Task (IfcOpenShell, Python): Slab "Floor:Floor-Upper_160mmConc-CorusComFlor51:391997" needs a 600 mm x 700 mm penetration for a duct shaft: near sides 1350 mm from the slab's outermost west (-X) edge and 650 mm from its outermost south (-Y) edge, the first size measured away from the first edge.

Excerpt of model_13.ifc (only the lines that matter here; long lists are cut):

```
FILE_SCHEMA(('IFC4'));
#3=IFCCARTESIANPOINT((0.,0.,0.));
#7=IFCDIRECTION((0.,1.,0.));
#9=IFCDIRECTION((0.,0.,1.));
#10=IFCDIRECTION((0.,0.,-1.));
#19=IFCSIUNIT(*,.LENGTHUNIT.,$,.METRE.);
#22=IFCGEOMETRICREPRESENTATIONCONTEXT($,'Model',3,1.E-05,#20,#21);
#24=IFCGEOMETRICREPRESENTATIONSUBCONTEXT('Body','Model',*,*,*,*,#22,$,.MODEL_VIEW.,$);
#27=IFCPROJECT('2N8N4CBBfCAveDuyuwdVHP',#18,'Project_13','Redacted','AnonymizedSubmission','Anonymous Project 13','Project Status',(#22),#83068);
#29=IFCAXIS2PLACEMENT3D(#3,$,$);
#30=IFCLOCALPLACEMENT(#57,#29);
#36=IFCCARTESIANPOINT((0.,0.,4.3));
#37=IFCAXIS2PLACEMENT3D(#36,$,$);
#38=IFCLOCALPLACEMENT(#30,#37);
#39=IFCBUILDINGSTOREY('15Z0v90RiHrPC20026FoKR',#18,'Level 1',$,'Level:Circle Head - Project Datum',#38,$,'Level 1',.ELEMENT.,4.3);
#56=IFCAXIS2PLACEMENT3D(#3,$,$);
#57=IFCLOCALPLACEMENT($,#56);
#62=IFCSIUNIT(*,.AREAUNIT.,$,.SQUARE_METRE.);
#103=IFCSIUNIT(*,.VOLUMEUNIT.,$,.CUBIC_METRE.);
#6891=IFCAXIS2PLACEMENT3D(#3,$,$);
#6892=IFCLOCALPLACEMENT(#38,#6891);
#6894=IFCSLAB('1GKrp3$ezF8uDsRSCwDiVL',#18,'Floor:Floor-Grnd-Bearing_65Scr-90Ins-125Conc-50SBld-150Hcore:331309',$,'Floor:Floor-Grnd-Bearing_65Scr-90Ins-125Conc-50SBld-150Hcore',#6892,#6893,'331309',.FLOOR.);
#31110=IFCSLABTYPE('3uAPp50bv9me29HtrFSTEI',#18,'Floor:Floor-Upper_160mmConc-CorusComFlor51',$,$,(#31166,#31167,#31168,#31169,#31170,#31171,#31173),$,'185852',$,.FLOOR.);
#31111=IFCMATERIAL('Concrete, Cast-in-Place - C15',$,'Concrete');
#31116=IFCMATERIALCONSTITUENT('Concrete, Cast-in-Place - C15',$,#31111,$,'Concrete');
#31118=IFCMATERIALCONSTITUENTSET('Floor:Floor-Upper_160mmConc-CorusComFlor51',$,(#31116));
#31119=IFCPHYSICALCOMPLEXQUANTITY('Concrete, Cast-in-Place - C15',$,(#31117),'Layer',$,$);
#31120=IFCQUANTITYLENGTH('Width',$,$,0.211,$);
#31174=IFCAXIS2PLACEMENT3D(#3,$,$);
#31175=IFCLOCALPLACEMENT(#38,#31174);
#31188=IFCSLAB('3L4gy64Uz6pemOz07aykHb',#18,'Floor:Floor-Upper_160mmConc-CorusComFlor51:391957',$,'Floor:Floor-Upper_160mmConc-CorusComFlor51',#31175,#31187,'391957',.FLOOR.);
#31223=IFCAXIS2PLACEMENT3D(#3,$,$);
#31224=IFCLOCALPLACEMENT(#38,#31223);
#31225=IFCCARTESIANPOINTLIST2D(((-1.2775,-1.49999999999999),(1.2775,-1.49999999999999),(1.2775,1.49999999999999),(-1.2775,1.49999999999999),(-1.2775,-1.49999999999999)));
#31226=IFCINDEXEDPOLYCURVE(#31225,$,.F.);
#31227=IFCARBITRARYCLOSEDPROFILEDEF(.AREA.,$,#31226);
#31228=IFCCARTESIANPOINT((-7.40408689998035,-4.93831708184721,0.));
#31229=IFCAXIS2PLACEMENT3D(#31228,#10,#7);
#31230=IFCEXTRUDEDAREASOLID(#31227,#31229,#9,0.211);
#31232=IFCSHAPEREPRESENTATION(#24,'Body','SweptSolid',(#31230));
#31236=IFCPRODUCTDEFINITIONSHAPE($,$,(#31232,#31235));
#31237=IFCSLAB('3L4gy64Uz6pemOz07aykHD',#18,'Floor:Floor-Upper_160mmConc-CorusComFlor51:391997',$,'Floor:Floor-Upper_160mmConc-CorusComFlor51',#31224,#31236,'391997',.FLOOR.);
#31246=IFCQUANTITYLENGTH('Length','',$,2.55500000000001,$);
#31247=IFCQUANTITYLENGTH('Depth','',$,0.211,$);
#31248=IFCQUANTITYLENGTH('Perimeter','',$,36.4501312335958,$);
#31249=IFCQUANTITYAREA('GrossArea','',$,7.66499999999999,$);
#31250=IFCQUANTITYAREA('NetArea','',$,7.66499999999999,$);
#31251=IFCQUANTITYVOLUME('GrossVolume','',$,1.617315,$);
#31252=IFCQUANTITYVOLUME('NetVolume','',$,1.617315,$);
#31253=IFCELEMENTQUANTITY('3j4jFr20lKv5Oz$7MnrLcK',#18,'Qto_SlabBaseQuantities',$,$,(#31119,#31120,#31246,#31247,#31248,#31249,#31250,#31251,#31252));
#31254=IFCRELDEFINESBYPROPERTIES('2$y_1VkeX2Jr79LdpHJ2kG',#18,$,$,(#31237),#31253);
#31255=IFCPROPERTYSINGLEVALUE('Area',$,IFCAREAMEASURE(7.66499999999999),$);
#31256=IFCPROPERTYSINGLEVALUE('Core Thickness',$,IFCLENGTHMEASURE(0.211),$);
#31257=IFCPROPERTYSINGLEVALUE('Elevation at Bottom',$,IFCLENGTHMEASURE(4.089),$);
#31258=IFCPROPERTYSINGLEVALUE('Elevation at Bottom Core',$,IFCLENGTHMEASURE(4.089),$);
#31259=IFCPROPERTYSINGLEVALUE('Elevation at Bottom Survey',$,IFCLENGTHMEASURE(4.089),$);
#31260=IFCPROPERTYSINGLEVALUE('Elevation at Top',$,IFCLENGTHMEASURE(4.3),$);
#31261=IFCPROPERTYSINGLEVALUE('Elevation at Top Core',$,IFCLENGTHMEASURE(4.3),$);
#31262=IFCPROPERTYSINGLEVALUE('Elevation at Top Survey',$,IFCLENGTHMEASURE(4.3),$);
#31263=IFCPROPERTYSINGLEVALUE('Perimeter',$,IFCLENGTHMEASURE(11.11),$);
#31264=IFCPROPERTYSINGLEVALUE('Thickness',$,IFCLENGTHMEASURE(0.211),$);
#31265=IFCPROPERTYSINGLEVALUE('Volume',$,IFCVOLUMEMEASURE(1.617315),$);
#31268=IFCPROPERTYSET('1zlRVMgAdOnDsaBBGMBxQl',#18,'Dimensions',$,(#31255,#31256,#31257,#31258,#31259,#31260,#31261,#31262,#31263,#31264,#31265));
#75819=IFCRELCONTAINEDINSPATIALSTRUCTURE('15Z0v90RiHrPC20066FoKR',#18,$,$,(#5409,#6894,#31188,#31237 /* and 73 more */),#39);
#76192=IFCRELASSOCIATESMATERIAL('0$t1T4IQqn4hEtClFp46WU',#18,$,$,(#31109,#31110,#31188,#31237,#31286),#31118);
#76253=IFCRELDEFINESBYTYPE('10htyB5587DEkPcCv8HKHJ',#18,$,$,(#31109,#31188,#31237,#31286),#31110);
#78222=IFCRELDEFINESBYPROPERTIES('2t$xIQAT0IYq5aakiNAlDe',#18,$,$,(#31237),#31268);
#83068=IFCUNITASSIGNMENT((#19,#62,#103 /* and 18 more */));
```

```python
import numpy as np
import ifcopenshell
import ifcopenshell.api.feature
import ifcopenshell.api.geometry
import ifcopenshell.api.pset
import ifcopenshell.api.root
import ifcopenshell.geom
import ifcopenshell.util.element
import ifcopenshell.util.placement
import ifcopenshell.util.representation
import ifcopenshell.util.shape
import ifcopenshell.util.unit

model = ifcopenshell.open("model_13.ifc")
unit_scale = ifcopenshell.util.unit.calculate_unit_scale(model)
area_scale = ifcopenshell.util.unit.calculate_unit_scale(model, "AREAUNIT")
volume_scale = ifcopenshell.util.unit.calculate_unit_scale(model, "VOLUMEUNIT")
settings = ifcopenshell.geom.settings()


def volume(element):
    """Net volume in cubic metres, openings subtracted."""
    shape = ifcopenshell.geom.create_shape(settings, element)
    return ifcopenshell.util.shape.get_volume(shape.geometry)


slab = model.by_id(31237)
before = volume(slab)

# Extent in the slab's own axes, in metres. The edges named are its -X and -Y sides.
slab_shape = ifcopenshell.geom.create_shape(settings, slab)
vertices = ifcopenshell.util.shape.get_vertices(slab_shape.geometry)
x_min, y_min, bottom = vertices.min(axis=0)
top = vertices[:, 2].max()

opening = ifcopenshell.api.root.create_entity(model, ifc_class="IfcOpeningElement", name="Duct shaft opening", predefined_type="OPENING")
context = ifcopenshell.util.representation.get_context(model, "Model", "Body", "MODEL_VIEW")
width, depth = 0.6, 0.7
outline = [(0.0, 0.0), (width, 0.0), (width, depth), (0.0, depth), (0.0, 0.0)]
# Overshoot both faces by 50 mm so the cut is clean.
shape = ifcopenshell.api.geometry.add_slab_representation(
    model, context=context, depth=top - bottom + 0.1, polyline=outline
)
ifcopenshell.api.geometry.assign_representation(model, product=opening, representation=shape)

matrix = ifcopenshell.util.placement.get_local_placement(slab.ObjectPlacement)
matrix[:, 3] = matrix @ np.append(np.array([x_min + 1.35, y_min + 0.65, bottom - 0.05]) / unit_scale, 1.0)
ifcopenshell.api.geometry.edit_object_placement(model, product=opening, matrix=matrix, is_si=False)
ifcopenshell.api.feature.add_feature(model, feature=opening, element=slab)

after = volume(slab)

# Update the slab's stored quantities.
qto = model.by_id(ifcopenshell.util.element.get_pset(slab, "Qto_SlabBaseQuantities", should_inherit=False)["id"])
ifcopenshell.api.pset.edit_qto(model, qto=qto, properties={
    "NetArea": after / (top - bottom) / area_scale,
    "NetVolume": after / volume_scale,
})
pset = model.by_id(ifcopenshell.util.element.get_pset(slab, "Dimensions", should_inherit=False)["id"])
ifcopenshell.api.pset.edit_pset(model, pset=pset, properties={
    "Area": model.create_entity("IfcAreaMeasure", after / (top - bottom) / area_scale),
    "Volume": model.create_entity("IfcVolumeMeasure", after / volume_scale),
})

print(f"slab volume {before:.3f} -> {after:.3f} m3")

model.write("model_13-out.ifc")
```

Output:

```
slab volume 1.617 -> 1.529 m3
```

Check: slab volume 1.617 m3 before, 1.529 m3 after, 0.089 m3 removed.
